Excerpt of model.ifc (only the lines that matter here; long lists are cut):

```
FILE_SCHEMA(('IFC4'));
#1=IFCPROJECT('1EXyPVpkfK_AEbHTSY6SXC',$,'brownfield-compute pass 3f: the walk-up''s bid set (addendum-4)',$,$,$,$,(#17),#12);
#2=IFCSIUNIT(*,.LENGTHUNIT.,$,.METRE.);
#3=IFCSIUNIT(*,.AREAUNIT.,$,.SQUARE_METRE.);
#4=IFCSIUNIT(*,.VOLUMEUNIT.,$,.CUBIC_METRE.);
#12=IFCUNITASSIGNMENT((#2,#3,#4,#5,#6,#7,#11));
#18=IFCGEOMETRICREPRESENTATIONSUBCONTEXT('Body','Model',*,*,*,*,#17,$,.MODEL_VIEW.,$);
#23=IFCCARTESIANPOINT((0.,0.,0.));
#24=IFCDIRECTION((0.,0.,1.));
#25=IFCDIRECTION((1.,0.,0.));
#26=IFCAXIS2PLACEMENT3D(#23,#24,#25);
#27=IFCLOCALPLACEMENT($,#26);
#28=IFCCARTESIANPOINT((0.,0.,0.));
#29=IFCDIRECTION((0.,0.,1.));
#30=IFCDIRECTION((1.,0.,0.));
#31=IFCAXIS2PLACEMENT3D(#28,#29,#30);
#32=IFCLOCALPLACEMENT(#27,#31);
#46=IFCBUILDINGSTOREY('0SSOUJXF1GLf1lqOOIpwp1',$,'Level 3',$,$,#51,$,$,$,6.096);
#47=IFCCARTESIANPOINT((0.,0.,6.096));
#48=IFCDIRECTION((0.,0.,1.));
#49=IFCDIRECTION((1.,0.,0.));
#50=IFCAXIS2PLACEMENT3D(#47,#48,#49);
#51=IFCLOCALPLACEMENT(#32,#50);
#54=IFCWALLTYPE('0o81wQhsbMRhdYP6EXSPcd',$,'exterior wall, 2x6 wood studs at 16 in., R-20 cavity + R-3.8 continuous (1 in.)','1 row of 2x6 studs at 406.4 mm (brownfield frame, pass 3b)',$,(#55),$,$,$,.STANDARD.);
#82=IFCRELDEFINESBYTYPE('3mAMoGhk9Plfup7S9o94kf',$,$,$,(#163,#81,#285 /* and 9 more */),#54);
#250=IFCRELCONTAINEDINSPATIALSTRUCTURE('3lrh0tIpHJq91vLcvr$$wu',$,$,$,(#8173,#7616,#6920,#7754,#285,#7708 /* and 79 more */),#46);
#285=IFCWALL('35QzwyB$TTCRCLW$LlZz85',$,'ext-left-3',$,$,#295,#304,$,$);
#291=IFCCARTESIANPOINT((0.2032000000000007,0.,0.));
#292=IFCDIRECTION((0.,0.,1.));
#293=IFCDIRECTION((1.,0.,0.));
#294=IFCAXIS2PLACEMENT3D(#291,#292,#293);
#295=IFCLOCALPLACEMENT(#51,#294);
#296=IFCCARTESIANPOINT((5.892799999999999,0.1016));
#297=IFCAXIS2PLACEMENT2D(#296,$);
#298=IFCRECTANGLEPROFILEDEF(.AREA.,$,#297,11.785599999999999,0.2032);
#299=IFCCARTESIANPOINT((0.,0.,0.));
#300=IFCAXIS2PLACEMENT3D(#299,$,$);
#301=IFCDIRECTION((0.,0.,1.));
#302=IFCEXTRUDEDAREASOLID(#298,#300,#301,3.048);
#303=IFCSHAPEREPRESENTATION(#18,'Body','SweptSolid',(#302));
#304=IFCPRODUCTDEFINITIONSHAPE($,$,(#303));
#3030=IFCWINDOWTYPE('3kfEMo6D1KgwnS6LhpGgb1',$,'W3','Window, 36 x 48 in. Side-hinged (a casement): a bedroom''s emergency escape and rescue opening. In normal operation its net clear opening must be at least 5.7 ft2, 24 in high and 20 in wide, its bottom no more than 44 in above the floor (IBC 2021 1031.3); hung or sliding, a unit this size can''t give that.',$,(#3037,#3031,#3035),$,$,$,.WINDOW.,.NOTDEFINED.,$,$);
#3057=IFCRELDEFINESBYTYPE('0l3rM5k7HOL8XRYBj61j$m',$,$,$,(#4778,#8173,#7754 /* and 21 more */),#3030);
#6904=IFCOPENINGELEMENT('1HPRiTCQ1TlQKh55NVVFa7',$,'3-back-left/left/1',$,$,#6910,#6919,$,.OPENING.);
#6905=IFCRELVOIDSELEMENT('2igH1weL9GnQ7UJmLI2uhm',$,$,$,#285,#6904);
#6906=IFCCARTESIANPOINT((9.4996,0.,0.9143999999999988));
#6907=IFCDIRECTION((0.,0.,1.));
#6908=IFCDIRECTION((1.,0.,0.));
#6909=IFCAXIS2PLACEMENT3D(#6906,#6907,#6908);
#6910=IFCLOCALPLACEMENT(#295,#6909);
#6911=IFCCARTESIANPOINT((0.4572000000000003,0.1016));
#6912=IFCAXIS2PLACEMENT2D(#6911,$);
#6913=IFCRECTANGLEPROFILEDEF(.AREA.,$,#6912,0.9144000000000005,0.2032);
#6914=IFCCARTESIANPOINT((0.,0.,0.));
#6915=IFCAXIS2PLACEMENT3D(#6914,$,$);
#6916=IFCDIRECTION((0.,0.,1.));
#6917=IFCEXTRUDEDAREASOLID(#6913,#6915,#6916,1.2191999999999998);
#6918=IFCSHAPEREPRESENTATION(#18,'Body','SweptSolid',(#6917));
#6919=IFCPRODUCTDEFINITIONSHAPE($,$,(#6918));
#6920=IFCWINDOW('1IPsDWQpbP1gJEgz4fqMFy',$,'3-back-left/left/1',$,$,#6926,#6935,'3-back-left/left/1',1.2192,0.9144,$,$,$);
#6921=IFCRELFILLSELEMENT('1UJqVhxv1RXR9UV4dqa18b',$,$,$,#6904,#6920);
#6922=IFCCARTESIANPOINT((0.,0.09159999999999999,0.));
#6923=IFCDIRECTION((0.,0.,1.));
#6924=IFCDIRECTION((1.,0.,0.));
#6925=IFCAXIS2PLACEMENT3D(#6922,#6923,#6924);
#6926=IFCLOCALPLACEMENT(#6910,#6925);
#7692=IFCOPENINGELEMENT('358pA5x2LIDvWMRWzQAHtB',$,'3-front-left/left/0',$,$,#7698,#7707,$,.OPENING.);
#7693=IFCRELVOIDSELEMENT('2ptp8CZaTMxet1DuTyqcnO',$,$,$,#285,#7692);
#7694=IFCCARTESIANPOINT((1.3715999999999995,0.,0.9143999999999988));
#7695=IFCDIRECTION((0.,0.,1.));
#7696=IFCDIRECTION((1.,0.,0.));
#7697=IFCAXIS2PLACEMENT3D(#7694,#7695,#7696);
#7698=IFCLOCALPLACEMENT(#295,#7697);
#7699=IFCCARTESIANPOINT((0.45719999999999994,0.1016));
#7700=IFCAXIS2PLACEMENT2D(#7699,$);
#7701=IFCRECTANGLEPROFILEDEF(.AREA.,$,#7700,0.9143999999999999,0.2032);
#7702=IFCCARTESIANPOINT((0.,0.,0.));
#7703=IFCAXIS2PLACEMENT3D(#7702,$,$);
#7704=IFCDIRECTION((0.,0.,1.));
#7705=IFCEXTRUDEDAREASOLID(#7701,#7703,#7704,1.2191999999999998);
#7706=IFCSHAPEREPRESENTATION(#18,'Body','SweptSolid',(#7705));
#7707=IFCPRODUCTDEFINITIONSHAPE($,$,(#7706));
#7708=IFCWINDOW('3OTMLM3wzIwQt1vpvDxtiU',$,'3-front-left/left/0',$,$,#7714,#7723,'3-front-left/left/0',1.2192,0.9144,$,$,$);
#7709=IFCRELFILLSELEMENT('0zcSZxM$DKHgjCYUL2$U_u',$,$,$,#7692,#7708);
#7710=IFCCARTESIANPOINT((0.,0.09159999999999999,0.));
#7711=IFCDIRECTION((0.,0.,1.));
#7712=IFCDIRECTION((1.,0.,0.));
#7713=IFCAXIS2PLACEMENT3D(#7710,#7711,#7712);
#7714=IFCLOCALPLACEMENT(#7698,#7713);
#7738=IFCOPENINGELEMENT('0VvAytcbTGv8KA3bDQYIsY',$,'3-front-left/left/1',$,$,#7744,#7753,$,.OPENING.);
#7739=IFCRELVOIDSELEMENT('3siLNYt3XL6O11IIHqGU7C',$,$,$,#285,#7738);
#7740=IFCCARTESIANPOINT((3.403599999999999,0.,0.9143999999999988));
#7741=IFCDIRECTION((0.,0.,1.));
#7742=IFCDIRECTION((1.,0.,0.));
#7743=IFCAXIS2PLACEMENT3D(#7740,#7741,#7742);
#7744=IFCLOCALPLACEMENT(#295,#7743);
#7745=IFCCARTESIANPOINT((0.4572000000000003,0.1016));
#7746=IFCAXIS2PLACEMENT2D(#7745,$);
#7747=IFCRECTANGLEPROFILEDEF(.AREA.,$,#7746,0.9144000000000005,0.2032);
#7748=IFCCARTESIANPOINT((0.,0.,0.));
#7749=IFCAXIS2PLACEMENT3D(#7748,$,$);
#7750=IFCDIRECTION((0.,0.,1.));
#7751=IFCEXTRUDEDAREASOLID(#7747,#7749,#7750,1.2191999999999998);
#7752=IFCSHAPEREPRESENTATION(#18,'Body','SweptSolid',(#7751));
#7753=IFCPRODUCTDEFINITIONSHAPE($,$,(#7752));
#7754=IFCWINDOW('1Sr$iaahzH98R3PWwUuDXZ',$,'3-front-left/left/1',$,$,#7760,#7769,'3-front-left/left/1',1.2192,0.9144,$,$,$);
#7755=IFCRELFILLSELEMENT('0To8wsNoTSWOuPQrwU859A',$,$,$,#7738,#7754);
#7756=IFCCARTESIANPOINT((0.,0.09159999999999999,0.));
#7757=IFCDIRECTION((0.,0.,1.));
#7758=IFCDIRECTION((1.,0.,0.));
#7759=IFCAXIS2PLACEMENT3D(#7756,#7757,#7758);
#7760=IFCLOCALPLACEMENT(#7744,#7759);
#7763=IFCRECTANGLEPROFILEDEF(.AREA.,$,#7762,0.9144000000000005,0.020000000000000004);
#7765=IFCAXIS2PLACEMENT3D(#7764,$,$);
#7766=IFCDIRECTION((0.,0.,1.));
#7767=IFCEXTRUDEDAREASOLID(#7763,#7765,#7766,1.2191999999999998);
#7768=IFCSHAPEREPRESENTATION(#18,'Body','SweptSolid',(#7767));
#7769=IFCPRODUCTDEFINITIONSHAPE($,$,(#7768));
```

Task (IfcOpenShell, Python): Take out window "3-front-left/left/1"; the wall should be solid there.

```python
import ifcopenshell
import ifcopenshell.api.feature
import ifcopenshell.api.root
import ifcopenshell.geom
import ifcopenshell.util.shape

model = ifcopenshell.open("model.ifc")
settings = ifcopenshell.geom.settings()


def volume(element):
    """Net volume in cubic metres, openings subtracted."""
    shape = ifcopenshell.geom.create_shape(settings, element)
    return ifcopenshell.util.shape.get_volume(shape.geometry)


window = model.by_id(7754)
opening = window.FillsVoids[0].RelatingOpeningElement
wall = opening.VoidsElements[0].RelatingBuildingElement
before = volume(wall)

ifcopenshell.api.root.remove_product(model, product=window)
ifcopenshell.api.feature.remove_feature(model, feature=opening)

after = volume(wall)

print(f"wall volume {before:.3f} -> {after:.3f} m3")

model.write("model_v2.ifc")
```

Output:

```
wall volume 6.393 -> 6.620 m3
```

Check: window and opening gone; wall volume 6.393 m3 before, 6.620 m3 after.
